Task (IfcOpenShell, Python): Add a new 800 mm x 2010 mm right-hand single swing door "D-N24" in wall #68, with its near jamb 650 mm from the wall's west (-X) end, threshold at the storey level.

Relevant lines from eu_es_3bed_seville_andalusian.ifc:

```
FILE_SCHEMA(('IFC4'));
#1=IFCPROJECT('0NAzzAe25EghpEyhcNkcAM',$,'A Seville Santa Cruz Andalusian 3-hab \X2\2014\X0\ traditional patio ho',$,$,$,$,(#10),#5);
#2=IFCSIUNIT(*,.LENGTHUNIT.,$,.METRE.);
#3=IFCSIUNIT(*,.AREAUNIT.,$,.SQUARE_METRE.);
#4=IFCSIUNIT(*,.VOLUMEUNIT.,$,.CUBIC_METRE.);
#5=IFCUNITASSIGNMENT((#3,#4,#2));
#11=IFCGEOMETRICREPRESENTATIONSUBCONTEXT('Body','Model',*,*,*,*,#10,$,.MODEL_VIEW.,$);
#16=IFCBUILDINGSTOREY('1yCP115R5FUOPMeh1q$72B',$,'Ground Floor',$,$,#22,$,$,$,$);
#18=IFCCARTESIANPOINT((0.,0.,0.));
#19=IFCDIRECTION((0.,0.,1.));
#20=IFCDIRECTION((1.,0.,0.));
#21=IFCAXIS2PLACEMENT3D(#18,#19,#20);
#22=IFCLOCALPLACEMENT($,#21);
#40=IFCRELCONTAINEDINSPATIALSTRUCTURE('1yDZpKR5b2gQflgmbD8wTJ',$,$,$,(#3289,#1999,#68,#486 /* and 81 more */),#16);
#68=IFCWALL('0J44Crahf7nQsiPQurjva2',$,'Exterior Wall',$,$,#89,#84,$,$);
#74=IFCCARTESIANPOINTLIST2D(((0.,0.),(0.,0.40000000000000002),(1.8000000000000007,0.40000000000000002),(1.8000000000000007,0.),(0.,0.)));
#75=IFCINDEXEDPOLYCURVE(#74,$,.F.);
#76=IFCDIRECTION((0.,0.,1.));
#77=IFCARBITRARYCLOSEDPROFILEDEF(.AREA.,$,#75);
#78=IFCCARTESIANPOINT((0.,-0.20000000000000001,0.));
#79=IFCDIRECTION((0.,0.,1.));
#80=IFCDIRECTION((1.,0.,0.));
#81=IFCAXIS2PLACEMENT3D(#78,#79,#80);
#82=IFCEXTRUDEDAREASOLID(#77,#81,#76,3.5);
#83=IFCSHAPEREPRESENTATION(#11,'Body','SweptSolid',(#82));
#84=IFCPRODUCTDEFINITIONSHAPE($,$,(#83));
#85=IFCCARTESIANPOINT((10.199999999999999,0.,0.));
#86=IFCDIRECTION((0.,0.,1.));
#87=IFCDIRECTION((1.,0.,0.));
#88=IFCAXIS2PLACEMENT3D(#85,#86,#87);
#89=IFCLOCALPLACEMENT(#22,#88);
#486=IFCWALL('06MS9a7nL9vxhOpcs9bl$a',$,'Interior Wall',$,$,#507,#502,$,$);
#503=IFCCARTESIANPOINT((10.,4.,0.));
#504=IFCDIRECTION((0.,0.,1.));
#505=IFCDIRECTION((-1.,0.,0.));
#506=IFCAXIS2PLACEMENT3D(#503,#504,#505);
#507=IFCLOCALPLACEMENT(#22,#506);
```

```python
import numpy as np
import ifcopenshell
import ifcopenshell.api.feature
import ifcopenshell.api.geometry
import ifcopenshell.api.root
import ifcopenshell.api.spatial
import ifcopenshell.geom
import ifcopenshell.util.element
import ifcopenshell.util.placement
import ifcopenshell.util.representation
import ifcopenshell.util.shape
import ifcopenshell.util.unit

model = ifcopenshell.open("eu_es_3bed_seville_andalusian.ifc")
unit_scale = ifcopenshell.util.unit.calculate_unit_scale(model)
settings = ifcopenshell.geom.settings()


def volume(element):
    """Net volume in cubic metres, openings subtracted."""
    shape = ifcopenshell.geom.create_shape(settings, element)
    return ifcopenshell.util.shape.get_volume(shape.geometry)


wall = model.by_id(68)
storey = ifcopenshell.util.element.get_container(wall, ifc_class="IfcBuildingStorey")
context = ifcopenshell.util.representation.get_context(model, "Model", "Body", "MODEL_VIEW")
before = volume(wall)

width, height, from_end, sill = 0.8, 2.01, 0.65, 0.0  # metres

# The wall runs along its own X axis, and the end named is its -X end.
wall_shape = ifcopenshell.geom.create_shape(settings, wall)
x, y, z = ifcopenshell.util.shape.get_vertices(wall_shape.geometry).T
start = x.min() + from_end
face, thickness = float(y.min()), float(y.max() - y.min())
wall_matrix = ifcopenshell.util.placement.get_local_placement(wall.ObjectPlacement)
level = ifcopenshell.util.placement.get_local_placement(storey.ObjectPlacement)[2, 3]


def in_wall(x, y):
    """Placement at x, y metres in the wall's axes, at sill height."""
    matrix = wall_matrix.copy()
    matrix[:, 3] = wall_matrix @ np.array([x / unit_scale, y / unit_scale, 0.0, 1.0])
    matrix[2, 3] = level + sill / unit_scale
    return matrix


# Opening: a box that overshoots both wall faces by 50 mm.
opening = ifcopenshell.api.root.create_entity(model, ifc_class="IfcOpeningElement", predefined_type="OPENING")
box = ifcopenshell.api.geometry.add_wall_representation(
    model, context=context, length=width, height=height, thickness=thickness + 0.1
)
ifcopenshell.api.geometry.assign_representation(model, product=opening, representation=box)
ifcopenshell.api.geometry.edit_object_placement(model, product=opening, matrix=in_wall(start, face - 0.05), is_si=False)
ifcopenshell.api.feature.add_feature(model, feature=opening, element=wall)

door = ifcopenshell.api.root.create_entity(model, ifc_class="IfcDoor", name="D-N24", predefined_type="DOOR")
door.OverallWidth, door.OverallHeight = width / unit_scale, height / unit_scale
door.OperationType = "SINGLE_SWING_RIGHT"
body = ifcopenshell.api.geometry.add_door_representation(
    model,
    context=context,
    overall_width=door.OverallWidth,
    overall_height=door.OverallHeight,
    operation_type="SINGLE_SWING_RIGHT",
    lining_properties={"LiningDepth": thickness / unit_scale, "ThresholdDepth": thickness / unit_scale},
)
ifcopenshell.api.geometry.assign_representation(model, product=door, representation=body)
ifcopenshell.api.spatial.assign_container(model, products=[door], relating_structure=storey)
ifcopenshell.api.feature.add_filling(model, opening=opening, element=door)

# The lining spans the wall, so the door starts at the wall face.
ifcopenshell.api.geometry.edit_object_placement(model, product=door, matrix=in_wall(start, face), is_si=False)

after = volume(wall)

print(f"wall volume {before:.3f} -> {after:.3f} m3")

model.write("eu_es_3bed_seville_andalusian_updated.ifc")
```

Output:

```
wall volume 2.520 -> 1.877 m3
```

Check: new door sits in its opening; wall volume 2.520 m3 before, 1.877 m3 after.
